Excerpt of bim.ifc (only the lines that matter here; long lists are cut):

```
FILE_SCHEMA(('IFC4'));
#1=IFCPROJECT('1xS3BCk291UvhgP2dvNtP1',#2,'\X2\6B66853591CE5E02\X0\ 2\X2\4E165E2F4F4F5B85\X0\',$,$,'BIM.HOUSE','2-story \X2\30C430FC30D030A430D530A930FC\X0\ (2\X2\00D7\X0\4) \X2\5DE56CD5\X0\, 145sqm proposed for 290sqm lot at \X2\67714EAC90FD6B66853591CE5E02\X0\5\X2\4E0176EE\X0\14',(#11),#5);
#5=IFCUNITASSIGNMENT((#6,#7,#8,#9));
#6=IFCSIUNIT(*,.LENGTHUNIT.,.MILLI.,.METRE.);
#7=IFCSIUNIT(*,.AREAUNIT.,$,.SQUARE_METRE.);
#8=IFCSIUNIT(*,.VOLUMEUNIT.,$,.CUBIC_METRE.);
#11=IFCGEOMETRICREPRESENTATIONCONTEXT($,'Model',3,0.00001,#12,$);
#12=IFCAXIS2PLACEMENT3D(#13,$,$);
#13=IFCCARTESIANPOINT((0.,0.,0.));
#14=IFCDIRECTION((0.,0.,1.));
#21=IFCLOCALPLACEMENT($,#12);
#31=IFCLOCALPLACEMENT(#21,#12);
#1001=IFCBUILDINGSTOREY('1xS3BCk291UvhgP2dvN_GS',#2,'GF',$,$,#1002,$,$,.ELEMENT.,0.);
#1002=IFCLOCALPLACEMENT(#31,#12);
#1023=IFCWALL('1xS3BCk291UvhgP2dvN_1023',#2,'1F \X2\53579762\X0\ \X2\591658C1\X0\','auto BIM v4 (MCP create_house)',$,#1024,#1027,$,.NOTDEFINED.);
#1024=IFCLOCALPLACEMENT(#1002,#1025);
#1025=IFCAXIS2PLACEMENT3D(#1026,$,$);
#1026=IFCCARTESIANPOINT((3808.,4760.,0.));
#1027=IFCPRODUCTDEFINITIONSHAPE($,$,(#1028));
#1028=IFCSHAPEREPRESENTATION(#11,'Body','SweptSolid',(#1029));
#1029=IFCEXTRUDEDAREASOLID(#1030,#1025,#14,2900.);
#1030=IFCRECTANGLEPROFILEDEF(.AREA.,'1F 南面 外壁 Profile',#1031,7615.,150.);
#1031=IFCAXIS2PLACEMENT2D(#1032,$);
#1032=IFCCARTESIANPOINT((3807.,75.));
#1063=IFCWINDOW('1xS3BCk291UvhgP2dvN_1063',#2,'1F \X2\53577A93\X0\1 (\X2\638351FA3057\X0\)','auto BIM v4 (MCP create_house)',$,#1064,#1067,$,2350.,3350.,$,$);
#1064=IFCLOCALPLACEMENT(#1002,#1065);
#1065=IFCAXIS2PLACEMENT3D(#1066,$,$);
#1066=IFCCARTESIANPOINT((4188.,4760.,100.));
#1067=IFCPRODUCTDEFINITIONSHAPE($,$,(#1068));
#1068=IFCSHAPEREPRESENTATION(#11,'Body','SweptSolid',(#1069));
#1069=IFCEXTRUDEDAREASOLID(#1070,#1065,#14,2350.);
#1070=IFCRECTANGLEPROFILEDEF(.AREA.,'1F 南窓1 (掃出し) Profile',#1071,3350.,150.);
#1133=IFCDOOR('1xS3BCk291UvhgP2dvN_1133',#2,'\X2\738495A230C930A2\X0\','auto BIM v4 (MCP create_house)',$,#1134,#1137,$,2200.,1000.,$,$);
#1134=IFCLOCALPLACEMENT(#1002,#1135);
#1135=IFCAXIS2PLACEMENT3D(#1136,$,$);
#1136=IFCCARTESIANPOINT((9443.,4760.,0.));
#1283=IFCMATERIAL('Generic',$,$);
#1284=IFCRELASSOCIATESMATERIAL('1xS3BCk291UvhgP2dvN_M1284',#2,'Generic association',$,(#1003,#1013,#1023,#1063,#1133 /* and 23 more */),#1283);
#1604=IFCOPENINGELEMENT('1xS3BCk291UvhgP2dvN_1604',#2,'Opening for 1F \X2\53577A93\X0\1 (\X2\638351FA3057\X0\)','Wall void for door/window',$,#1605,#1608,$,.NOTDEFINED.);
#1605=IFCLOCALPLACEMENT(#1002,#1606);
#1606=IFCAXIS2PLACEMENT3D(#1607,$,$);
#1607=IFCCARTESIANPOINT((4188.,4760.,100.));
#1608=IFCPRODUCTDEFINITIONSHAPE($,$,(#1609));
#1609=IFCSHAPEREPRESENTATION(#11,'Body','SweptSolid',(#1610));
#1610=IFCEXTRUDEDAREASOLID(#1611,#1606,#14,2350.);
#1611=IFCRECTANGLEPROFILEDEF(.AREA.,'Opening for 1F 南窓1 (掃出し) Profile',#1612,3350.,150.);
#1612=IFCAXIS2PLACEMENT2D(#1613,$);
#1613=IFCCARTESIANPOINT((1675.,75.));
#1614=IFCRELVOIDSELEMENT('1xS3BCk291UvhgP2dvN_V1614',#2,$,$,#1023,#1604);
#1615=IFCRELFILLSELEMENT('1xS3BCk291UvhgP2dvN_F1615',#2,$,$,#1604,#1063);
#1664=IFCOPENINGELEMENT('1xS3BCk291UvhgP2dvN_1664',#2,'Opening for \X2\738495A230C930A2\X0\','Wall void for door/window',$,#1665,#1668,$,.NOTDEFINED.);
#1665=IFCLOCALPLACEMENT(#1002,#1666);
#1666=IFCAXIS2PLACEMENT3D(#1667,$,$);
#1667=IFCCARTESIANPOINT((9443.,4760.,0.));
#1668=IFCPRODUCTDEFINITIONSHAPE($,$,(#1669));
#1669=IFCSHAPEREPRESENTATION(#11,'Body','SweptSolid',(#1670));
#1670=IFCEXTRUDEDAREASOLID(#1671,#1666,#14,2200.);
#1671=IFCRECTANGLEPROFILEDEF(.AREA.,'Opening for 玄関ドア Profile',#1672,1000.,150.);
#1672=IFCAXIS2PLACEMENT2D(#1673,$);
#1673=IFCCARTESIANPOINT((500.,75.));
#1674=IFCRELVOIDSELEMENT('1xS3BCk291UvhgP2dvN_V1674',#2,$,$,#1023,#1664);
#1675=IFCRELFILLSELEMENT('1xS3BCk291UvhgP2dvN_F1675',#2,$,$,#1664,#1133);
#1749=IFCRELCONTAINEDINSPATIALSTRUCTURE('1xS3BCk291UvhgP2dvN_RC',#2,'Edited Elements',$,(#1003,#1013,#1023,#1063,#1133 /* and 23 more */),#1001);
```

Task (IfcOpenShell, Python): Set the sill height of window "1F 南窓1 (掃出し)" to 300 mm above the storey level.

```python
import numpy as np
import ifcopenshell
import ifcopenshell.api.geometry
import ifcopenshell.geom
import ifcopenshell.util.element
import ifcopenshell.util.placement
import ifcopenshell.util.shape
import ifcopenshell.util.unit

model = ifcopenshell.open("bim.ifc")
unit_scale = ifcopenshell.util.unit.calculate_unit_scale(model)

window = model.by_guid("1xS3BCk291UvhgP2dvN_1063")
opening = window.FillsVoids[0].RelatingOpeningElement
storey = ifcopenshell.util.element.get_container(window, ifc_class="IfcBuildingStorey")
level = ifcopenshell.util.placement.get_local_placement(storey.ObjectPlacement)[2, 3]

# The opening's origin need not be at the sill, so measure its lowest point.
shape = ifcopenshell.geom.create_shape(ifcopenshell.geom.settings(), opening)
bottom = ifcopenshell.util.shape.get_shape_bottom_elevation(shape, shape.geometry) / unit_scale
dz = level + 0.3 / unit_scale - bottom

shift = np.array([0.0, 0.0, dz])
# The window is not placed relative to its opening, so move both.
for product in (opening, window):
    matrix = ifcopenshell.util.placement.get_local_placement(product.ObjectPlacement)
    matrix[:3, 3] += shift
    ifcopenshell.api.geometry.edit_object_placement(model, product=product, matrix=matrix, is_si=False)

print(f"moved by {dz * unit_scale:+.3f} m")

model.write("bim_edited.ifc")
```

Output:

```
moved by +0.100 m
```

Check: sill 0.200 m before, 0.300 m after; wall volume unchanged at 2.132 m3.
